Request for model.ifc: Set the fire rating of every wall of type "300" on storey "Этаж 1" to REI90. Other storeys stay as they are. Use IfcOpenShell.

First a look at what the model holds.

```python
import ifcopenshell
import ifcopenshell.util.element

model = ifcopenshell.open("model.ifc")
print(model.schema)
storey = next(s for s in model.by_type("IfcBuildingStorey") if s.Name == "Этаж 1")
walls = [e for e in ifcopenshell.util.element.get_decomposition(storey) if e.is_a("IfcWall")]
seen = {}
for e in walls:
    element_type = ifcopenshell.util.element.get_type(e)
    key = (element_type.Name if element_type != e and element_type else None, ifcopenshell.util.element.get_pset(e, "Pset_WallCommon", "FireRating"))
    seen[key] = seen.get(key, 0) + 1
for (name, value), count in sorted(seen.items(), key=str):
    print(count, "x", name, "|", value)
```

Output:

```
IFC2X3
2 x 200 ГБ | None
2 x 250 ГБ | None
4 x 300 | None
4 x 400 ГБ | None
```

```python
import ifcopenshell
import ifcopenshell.api.pset
import ifcopenshell.util.element

model = ifcopenshell.open("model.ifc")

storey = next(s for s in model.by_type("IfcBuildingStorey") if s.Name == "Этаж 1")
walls = [e for e in ifcopenshell.util.element.get_decomposition(storey) if e.is_a("IfcWall")]

count = 0
for e in walls:
    element_type = ifcopenshell.util.element.get_type(e)
    if element_type in (None, e) or element_type.Name != "300":
        continue
    # add_pset returns the element's existing set when there is one.
    pset = ifcopenshell.api.pset.add_pset(model, product=e, name="Pset_WallCommon")
    ifcopenshell.api.pset.edit_pset(model, pset=pset, properties={"FireRating": "REI90"})
    count += 1

print(count, "walls updated")

model.write("model_v2.ifc")
```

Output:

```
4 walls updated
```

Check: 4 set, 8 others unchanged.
